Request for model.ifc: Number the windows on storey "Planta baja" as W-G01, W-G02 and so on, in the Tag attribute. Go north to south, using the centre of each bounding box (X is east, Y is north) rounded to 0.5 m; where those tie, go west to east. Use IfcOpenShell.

First a look at what the model holds.

```python
import ifcopenshell
import ifcopenshell.util.element
import ifcopenshell.util.placement

model = ifcopenshell.open("model.ifc")
print(model.schema)
storey = next(s for s in model.by_type("IfcBuildingStorey") if s.Name == "Planta baja")
windows = [e for e in ifcopenshell.util.element.get_decomposition(storey) if e.is_a("IfcWindow")]
for e in sorted(windows, key=lambda e: e.id()):
    origin = ifcopenshell.util.placement.get_local_placement(e.ObjectPlacement)[:3, 3]
    print(e.id(), e.Tag, e.Name, origin.round(2) + 0.0, sep=" | ")
```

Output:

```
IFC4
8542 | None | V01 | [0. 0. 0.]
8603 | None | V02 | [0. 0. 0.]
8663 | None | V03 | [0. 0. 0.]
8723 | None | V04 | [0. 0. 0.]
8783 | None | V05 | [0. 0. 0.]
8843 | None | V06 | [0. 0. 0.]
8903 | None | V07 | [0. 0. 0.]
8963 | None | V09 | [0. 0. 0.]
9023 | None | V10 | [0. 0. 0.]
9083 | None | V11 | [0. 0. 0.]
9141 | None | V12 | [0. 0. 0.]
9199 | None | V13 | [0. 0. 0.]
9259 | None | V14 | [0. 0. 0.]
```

```python
import ifcopenshell
import ifcopenshell.geom
import ifcopenshell.util.element
import ifcopenshell.util.shape

model = ifcopenshell.open("model.ifc")
settings = ifcopenshell.geom.settings()
settings.set("use-world-coords", True)


def centre(element):
    shape = ifcopenshell.geom.create_shape(settings, element)
    return ifcopenshell.util.shape.get_bbox_centroid(shape.geometry)


storey = next(s for s in model.by_type("IfcBuildingStorey") if s.Name == "Planta baja")
windows = [e for e in ifcopenshell.util.element.get_decomposition(storey) if e.is_a("IfcWindow")]

# Insertion points can sit at a corner or the storey origin, so sort by the geometry (in metres).
centres = {e: centre(e) for e in windows}
windows.sort(key=lambda e: (-round(centres[e][1] / 0.5), centres[e][0]))

for i, e in enumerate(windows, start=1):
    number = f"W-G{i:02d}"
    e.Tag = number
    print(e.id(), number)

model.write("model_v2.ifc")
```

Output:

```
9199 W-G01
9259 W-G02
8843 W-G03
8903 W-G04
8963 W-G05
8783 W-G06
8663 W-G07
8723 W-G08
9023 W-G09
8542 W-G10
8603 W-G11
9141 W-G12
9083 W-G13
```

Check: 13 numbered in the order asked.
